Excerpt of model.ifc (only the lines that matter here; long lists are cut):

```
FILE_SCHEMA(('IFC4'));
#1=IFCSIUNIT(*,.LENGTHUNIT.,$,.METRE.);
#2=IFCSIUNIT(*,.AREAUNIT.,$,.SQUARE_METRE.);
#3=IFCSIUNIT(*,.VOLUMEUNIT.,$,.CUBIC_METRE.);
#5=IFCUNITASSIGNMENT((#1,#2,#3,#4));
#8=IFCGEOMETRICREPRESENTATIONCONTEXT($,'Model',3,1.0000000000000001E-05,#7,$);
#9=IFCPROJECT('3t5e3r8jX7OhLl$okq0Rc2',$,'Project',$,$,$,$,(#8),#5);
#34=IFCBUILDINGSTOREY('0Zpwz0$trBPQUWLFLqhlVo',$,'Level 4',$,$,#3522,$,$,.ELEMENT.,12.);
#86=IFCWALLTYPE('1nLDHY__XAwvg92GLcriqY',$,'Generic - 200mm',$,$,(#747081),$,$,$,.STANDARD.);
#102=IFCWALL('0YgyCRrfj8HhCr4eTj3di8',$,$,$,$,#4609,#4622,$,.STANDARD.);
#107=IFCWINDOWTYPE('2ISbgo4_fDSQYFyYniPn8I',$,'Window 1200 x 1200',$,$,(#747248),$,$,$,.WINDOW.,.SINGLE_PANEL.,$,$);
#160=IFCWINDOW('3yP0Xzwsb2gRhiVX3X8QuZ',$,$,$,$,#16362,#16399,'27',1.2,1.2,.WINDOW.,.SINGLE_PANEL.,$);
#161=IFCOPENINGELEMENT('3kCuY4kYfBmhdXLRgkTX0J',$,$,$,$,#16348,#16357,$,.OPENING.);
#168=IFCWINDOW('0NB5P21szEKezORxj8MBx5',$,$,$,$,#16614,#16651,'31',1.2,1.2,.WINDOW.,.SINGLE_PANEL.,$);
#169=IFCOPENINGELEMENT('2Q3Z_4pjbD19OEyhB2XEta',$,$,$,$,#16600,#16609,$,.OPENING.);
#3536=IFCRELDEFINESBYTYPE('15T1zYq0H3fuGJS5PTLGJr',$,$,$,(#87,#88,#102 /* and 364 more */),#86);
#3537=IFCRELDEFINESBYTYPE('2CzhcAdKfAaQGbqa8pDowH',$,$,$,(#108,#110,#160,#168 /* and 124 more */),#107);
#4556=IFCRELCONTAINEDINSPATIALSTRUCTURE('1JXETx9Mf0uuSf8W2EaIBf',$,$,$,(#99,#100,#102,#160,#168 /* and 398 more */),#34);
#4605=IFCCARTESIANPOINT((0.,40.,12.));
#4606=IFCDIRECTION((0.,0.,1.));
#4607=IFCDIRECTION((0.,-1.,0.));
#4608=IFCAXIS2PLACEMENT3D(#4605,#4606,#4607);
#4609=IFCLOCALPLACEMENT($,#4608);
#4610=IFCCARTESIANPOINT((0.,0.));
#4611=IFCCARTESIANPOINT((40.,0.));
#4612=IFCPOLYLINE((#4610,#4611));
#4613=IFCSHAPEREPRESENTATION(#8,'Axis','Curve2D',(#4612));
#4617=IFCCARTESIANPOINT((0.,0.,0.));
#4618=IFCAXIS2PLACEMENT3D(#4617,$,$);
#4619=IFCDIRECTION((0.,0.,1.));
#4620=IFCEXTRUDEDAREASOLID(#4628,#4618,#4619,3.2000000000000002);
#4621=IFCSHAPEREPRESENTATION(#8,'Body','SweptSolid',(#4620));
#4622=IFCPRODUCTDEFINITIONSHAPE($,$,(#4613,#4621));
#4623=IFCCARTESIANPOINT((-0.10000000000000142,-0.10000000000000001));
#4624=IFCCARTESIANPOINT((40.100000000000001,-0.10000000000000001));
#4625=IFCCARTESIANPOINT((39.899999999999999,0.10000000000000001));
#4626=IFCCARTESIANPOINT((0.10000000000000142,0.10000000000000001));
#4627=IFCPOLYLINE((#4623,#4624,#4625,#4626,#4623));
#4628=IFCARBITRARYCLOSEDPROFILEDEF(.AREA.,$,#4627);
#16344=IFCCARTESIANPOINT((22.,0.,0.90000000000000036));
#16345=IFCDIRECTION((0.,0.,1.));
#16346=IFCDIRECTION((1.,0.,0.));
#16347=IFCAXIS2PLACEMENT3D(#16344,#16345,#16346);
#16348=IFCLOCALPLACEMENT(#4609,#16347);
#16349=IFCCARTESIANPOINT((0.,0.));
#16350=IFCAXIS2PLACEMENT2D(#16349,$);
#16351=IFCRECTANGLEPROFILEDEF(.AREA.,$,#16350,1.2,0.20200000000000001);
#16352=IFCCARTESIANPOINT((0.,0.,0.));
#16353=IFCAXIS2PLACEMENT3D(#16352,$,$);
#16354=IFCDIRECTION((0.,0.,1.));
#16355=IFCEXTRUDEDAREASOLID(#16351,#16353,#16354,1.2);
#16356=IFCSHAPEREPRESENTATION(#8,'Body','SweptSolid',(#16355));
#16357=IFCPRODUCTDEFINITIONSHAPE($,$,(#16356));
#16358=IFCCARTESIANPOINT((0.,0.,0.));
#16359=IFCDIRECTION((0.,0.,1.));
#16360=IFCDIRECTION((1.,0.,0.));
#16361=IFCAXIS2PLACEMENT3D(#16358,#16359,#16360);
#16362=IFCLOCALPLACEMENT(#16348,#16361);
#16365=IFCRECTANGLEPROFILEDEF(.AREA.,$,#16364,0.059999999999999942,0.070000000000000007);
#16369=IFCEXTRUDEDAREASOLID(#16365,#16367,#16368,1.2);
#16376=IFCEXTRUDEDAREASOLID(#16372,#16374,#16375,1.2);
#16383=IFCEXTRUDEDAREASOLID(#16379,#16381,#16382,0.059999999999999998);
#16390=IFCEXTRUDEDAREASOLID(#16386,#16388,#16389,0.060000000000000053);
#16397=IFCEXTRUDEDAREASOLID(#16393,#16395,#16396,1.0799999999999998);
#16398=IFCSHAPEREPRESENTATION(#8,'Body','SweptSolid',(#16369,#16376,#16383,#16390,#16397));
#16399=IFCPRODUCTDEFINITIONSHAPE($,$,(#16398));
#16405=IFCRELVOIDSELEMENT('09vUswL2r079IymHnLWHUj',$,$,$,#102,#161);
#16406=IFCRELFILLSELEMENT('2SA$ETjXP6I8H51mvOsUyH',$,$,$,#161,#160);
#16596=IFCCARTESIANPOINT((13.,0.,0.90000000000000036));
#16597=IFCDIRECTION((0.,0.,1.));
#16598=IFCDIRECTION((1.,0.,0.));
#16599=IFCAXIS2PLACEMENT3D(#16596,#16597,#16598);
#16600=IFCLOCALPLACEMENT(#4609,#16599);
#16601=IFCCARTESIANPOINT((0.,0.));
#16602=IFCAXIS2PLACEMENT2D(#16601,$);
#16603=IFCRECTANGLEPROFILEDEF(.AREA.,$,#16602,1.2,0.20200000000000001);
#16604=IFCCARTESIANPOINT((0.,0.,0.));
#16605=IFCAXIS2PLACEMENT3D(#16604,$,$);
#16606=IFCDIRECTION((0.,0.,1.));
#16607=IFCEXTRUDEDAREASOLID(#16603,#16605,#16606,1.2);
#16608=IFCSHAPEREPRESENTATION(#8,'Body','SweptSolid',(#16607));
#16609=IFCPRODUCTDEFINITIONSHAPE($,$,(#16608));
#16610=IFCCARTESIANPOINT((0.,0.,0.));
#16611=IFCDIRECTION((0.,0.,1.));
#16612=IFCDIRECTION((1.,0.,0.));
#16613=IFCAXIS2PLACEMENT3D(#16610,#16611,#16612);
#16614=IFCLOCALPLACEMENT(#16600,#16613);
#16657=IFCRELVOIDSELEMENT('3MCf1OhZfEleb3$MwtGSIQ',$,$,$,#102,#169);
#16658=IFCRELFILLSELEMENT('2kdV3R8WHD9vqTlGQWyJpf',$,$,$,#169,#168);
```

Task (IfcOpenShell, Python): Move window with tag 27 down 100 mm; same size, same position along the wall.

```python
import numpy as np
import ifcopenshell
import ifcopenshell.api.geometry
import ifcopenshell.util.placement
import ifcopenshell.util.unit

model = ifcopenshell.open("model.ifc")
unit_scale = ifcopenshell.util.unit.calculate_unit_scale(model)

window = model.by_guid("3yP0Xzwsb2gRhiVX3X8QuZ")
opening = window.FillsVoids[0].RelatingOpeningElement
dz = -0.1 / unit_scale

shift = np.array([0.0, 0.0, dz])
# The window is placed relative to its opening, so it follows when the opening moves.
matrix = ifcopenshell.util.placement.get_local_placement(opening.ObjectPlacement)
matrix[:3, 3] += shift
ifcopenshell.api.geometry.edit_object_placement(
    model, product=opening, matrix=matrix, is_si=False, should_transform_children=True
)

print(f"moved by {dz * unit_scale:+.3f} m")

model.write("model_rev.ifc")
```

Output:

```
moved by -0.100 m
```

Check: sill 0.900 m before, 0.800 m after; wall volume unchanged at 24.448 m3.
